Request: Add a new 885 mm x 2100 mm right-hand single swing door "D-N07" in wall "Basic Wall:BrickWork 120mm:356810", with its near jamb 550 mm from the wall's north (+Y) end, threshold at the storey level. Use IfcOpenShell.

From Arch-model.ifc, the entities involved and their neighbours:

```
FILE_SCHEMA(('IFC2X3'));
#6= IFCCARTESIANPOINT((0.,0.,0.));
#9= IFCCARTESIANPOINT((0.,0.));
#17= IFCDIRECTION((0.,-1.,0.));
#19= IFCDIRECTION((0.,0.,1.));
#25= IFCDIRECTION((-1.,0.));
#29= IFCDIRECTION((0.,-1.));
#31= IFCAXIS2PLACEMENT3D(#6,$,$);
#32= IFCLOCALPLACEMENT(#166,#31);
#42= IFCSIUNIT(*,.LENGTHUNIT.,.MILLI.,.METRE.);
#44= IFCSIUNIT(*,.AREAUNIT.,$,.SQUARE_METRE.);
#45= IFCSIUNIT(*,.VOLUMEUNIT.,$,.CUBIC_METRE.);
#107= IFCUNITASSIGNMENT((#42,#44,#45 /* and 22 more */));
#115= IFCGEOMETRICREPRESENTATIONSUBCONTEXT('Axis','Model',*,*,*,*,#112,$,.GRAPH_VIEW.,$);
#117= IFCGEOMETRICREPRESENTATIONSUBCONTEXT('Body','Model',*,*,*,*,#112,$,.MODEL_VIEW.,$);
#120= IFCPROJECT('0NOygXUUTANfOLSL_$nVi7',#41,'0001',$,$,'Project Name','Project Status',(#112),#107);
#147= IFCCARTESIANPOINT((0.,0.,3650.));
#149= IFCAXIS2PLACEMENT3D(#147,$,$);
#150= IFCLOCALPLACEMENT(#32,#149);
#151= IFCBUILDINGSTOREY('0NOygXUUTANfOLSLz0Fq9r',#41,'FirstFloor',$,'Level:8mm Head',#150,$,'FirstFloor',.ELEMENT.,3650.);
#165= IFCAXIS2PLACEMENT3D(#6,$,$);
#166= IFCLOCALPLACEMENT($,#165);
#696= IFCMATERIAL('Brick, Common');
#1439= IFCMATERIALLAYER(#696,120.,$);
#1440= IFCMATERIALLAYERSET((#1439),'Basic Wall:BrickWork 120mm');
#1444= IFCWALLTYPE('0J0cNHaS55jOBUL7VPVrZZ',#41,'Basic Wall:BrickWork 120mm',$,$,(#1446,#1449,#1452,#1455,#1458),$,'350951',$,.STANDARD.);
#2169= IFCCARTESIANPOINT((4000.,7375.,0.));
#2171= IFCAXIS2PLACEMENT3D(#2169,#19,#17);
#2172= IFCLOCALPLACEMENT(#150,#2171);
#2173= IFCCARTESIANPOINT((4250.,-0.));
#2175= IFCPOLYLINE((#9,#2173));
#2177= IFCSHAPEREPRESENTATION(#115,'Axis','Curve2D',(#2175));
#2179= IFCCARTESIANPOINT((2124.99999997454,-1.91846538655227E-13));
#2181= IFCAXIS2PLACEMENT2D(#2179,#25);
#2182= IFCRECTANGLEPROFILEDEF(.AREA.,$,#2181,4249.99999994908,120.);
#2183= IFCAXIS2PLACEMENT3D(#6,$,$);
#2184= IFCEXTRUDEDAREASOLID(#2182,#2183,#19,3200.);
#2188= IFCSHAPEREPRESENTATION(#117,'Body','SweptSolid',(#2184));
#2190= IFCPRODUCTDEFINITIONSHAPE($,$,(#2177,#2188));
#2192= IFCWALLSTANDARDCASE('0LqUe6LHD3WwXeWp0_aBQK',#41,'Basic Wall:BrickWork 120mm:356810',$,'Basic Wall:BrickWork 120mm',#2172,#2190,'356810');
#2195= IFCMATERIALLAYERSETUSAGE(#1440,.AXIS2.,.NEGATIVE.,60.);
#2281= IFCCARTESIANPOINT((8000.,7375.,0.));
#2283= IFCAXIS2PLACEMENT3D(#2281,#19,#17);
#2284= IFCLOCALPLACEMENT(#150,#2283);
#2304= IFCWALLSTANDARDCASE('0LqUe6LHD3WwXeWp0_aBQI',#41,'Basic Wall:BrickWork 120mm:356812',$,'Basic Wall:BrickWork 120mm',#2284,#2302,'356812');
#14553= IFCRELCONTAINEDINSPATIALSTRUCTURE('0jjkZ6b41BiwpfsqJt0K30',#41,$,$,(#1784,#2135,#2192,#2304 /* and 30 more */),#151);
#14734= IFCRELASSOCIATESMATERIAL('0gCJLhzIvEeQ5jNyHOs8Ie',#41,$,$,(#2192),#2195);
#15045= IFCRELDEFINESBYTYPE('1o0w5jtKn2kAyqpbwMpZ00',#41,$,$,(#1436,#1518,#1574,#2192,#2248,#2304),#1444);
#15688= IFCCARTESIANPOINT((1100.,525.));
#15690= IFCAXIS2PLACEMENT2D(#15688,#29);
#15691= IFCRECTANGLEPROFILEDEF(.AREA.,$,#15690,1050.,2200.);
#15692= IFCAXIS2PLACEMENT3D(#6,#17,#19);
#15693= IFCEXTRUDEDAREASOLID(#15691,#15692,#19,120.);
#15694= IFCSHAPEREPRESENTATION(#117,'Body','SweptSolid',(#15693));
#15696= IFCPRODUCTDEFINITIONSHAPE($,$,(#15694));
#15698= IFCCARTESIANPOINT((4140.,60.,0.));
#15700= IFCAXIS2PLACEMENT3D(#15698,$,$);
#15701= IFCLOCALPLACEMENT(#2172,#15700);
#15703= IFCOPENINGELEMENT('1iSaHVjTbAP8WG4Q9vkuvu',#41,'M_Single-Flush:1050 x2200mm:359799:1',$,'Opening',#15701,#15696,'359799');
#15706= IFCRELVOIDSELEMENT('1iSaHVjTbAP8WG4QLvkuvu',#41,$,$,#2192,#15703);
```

```python
import numpy as np
import ifcopenshell
import ifcopenshell.api.feature
import ifcopenshell.api.geometry
import ifcopenshell.api.root
import ifcopenshell.api.spatial
import ifcopenshell.api.type
import ifcopenshell.geom
import ifcopenshell.util.element
import ifcopenshell.util.placement
import ifcopenshell.util.representation
import ifcopenshell.util.shape
import ifcopenshell.util.unit

model = ifcopenshell.open("Arch-model.ifc")
unit_scale = ifcopenshell.util.unit.calculate_unit_scale(model)
settings = ifcopenshell.geom.settings()


def volume(element):
    """Net volume in cubic metres, openings subtracted."""
    shape = ifcopenshell.geom.create_shape(settings, element)
    return ifcopenshell.util.shape.get_volume(shape.geometry)


wall = model.by_guid("0LqUe6LHD3WwXeWp0_aBQK")
storey = ifcopenshell.util.element.get_container(wall, ifc_class="IfcBuildingStorey")
context = ifcopenshell.util.representation.get_context(model, "Model", "Body", "MODEL_VIEW")
before = volume(wall)

width, height, from_end, sill = 0.885, 2.1, 0.55, 0.0  # metres

# The wall runs along its own X axis, and the end named is its -X end.
wall_shape = ifcopenshell.geom.create_shape(settings, wall)
x, y, z = ifcopenshell.util.shape.get_vertices(wall_shape.geometry).T
start = x.min() + from_end
face, thickness = float(y.min()), float(y.max() - y.min())
wall_matrix = ifcopenshell.util.placement.get_local_placement(wall.ObjectPlacement)
level = ifcopenshell.util.placement.get_local_placement(storey.ObjectPlacement)[2, 3]


def in_wall(x, y):
    """Placement at x, y metres in the wall's axes, at sill height."""
    matrix = wall_matrix.copy()
    matrix[:, 3] = wall_matrix @ np.array([x / unit_scale, y / unit_scale, 0.0, 1.0])
    matrix[2, 3] = level + sill / unit_scale
    return matrix


# Opening: a box that overshoots both wall faces by 50 mm.
opening = ifcopenshell.api.root.create_entity(model, ifc_class="IfcOpeningElement")
box = ifcopenshell.api.geometry.add_wall_representation(
    model, context=context, length=width, height=height, thickness=thickness + 0.1
)
ifcopenshell.api.geometry.assign_representation(model, product=opening, representation=box)
ifcopenshell.api.geometry.edit_object_placement(model, product=opening, matrix=in_wall(start, face - 0.05), is_si=False)
ifcopenshell.api.feature.add_feature(model, feature=opening, element=wall)

door = ifcopenshell.api.root.create_entity(model, ifc_class="IfcDoor", name="D-N07")
door.OverallWidth, door.OverallHeight = width / unit_scale, height / unit_scale
body = ifcopenshell.api.geometry.add_door_representation(
    model,
    context=context,
    overall_width=door.OverallWidth,
    overall_height=door.OverallHeight,
    operation_type="SINGLE_SWING_RIGHT",
    lining_properties={"LiningDepth": thickness / unit_scale, "ThresholdDepth": thickness / unit_scale},
)
ifcopenshell.api.geometry.assign_representation(model, product=door, representation=body)
ifcopenshell.api.spatial.assign_container(model, products=[door], relating_structure=storey)
fills = ifcopenshell.api.feature.add_filling(model, opening=opening, element=door)
fills.OwnerHistory = door.OwnerHistory  # required in IFC2X3

# IFC2X3 keeps the operation on the door style.
style = ifcopenshell.api.root.create_entity(model, ifc_class="IfcDoorStyle", name="D-N07")
style.OperationType, style.ConstructionType = "SINGLE_SWING_RIGHT", "NOTDEFINED"
style.ParameterTakesPrecedence = style.Sizeable = False
ifcopenshell.api.type.assign_type(model, related_objects=[door], relating_type=style)

# The lining spans the wall, so the door starts at the wall face.
ifcopenshell.api.geometry.edit_object_placement(model, product=door, matrix=in_wall(start, face), is_si=False)

after = volume(wall)

print(f"wall volume {before:.3f} -> {after:.3f} m3")

model.write("Arch-model-out.ifc")
```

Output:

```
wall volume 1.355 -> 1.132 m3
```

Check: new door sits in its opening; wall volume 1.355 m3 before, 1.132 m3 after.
